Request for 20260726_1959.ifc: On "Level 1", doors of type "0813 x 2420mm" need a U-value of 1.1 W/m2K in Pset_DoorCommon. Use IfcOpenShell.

First a look at what the model holds.

```python
import ifcopenshell
import ifcopenshell.util.element

model = ifcopenshell.open("20260726_1959.ifc")
print(model.schema)
storey = next(s for s in model.by_type("IfcBuildingStorey") if s.Name == "Level 1")
doors = [e for e in ifcopenshell.util.element.get_decomposition(storey) if e.is_a("IfcDoor")]
seen = {}
for e in doors:
    element_type = ifcopenshell.util.element.get_type(e)
    key = (element_type.Name if element_type != e and element_type else None, ifcopenshell.util.element.get_pset(e, "Pset_DoorCommon", "ThermalTransmittance"))
    seen[key] = seen.get(key, 0) + 1
for (name, value), count in sorted(seen.items(), key=str):
    print(count, "x", name, "|", value)
```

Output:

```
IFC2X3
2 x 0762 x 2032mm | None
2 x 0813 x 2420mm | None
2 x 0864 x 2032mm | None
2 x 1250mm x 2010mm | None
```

```python
import ifcopenshell
import ifcopenshell.api.pset
import ifcopenshell.util.element

model = ifcopenshell.open("20260726_1959.ifc")

storey = next(s for s in model.by_type("IfcBuildingStorey") if s.Name == "Level 1")
doors = [e for e in ifcopenshell.util.element.get_decomposition(storey) if e.is_a("IfcDoor")]

count = 0
for e in doors:
    element_type = ifcopenshell.util.element.get_type(e)
    if element_type in (None, e) or element_type.Name != "0813 x 2420mm":
        continue
    # add_pset returns the element's existing set when there is one.
    pset = ifcopenshell.api.pset.add_pset(model, product=e, name="Pset_DoorCommon")
    ifcopenshell.api.pset.edit_pset(model, pset=pset, properties={"ThermalTransmittance": 1.1})
    count += 1

print(count, "doors updated")

model.write("20260726_1959_rev.ifc")
```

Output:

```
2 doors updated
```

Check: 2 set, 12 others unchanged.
